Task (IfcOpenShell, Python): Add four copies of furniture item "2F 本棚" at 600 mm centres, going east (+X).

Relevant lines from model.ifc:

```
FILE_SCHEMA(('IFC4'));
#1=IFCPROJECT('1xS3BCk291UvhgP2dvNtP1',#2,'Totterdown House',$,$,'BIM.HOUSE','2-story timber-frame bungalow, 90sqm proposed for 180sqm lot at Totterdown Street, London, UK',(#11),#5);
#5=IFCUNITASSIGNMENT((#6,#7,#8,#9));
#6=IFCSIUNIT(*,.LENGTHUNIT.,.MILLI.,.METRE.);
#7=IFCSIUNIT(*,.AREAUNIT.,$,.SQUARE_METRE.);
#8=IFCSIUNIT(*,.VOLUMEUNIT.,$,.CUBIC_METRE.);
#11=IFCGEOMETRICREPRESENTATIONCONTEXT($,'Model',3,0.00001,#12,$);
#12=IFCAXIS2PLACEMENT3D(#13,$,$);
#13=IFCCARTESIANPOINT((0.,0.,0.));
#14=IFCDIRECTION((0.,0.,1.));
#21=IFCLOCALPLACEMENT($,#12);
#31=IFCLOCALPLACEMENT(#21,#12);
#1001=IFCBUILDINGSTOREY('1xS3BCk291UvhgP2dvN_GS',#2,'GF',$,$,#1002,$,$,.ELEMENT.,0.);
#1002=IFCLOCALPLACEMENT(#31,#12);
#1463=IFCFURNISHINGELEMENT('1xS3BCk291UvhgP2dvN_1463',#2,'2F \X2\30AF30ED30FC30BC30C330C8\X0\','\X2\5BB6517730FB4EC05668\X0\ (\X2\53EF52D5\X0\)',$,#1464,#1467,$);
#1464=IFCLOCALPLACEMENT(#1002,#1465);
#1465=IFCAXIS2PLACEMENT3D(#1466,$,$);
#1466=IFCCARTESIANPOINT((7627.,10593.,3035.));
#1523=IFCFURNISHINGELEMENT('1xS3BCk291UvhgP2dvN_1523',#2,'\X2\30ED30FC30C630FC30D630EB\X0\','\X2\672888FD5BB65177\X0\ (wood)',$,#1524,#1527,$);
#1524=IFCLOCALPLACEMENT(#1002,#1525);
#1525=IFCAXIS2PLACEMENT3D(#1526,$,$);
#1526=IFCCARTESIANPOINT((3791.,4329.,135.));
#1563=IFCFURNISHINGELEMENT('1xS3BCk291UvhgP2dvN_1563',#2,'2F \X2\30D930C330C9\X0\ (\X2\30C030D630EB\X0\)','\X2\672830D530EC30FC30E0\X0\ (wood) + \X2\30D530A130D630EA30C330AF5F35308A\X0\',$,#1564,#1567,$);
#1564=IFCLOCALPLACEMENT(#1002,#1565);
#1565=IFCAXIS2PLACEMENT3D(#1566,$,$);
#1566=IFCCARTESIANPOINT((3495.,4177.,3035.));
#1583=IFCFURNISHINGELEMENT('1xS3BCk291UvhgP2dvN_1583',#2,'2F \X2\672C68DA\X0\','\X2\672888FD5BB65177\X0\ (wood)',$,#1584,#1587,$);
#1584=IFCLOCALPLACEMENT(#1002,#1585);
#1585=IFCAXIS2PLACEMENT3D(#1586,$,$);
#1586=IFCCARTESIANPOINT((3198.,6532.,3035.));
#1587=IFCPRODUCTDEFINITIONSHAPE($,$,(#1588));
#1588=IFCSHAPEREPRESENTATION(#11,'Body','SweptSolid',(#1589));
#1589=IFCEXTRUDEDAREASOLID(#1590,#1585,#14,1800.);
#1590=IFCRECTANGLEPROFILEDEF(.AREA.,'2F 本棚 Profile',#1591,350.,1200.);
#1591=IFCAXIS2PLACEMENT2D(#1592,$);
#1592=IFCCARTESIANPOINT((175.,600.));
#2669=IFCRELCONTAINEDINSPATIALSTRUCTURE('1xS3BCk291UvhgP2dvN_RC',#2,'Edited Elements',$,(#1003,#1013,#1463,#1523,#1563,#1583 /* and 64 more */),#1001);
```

```python
import numpy as np
import ifcopenshell
import ifcopenshell.api.geometry
import ifcopenshell.api.root
import ifcopenshell.util.element
import ifcopenshell.util.placement
import ifcopenshell.util.unit

model = ifcopenshell.open("model.ifc")
unit_scale = ifcopenshell.util.unit.calculate_unit_scale(model)


def reuse_history(source, copy):
    """copy_class also copies each property set's owner history, people and application; keep the originals."""
    for rel in copy.IsDefinedBy:
        if rel.is_a("IfcRelDefinesByProperties") and (history := rel.RelatingPropertyDefinition.OwnerHistory):
            rel.RelatingPropertyDefinition.OwnerHistory = source.OwnerHistory
            ifcopenshell.util.element.remove_deep2(model, history)


source = model.by_guid("1xS3BCk291UvhgP2dvN_1583")
base = ifcopenshell.util.placement.get_local_placement(source.ObjectPlacement)
step = np.array([1.0, 0.0, 0.0]) * 0.6 / unit_scale

for i in range(1, 5):
    copy = ifcopenshell.api.root.copy_class(model, product=source)
    copy.Representation = ifcopenshell.util.element.copy_deep(
        model, source.Representation, exclude=["IfcGeometricRepresentationContext", "IfcRepresentationMap"]
    )
    reuse_history(source, copy)
    matrix = base.copy()
    matrix[:3, 3] += i * step
    print("added at", matrix[:3, 3].round(3) + 0.0)
    ifcopenshell.api.geometry.edit_object_placement(model, product=copy, matrix=matrix, is_si=False)

model.write("model_updated.ifc")
```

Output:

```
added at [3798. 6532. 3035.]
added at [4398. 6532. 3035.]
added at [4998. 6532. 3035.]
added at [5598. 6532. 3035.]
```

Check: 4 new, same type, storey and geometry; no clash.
